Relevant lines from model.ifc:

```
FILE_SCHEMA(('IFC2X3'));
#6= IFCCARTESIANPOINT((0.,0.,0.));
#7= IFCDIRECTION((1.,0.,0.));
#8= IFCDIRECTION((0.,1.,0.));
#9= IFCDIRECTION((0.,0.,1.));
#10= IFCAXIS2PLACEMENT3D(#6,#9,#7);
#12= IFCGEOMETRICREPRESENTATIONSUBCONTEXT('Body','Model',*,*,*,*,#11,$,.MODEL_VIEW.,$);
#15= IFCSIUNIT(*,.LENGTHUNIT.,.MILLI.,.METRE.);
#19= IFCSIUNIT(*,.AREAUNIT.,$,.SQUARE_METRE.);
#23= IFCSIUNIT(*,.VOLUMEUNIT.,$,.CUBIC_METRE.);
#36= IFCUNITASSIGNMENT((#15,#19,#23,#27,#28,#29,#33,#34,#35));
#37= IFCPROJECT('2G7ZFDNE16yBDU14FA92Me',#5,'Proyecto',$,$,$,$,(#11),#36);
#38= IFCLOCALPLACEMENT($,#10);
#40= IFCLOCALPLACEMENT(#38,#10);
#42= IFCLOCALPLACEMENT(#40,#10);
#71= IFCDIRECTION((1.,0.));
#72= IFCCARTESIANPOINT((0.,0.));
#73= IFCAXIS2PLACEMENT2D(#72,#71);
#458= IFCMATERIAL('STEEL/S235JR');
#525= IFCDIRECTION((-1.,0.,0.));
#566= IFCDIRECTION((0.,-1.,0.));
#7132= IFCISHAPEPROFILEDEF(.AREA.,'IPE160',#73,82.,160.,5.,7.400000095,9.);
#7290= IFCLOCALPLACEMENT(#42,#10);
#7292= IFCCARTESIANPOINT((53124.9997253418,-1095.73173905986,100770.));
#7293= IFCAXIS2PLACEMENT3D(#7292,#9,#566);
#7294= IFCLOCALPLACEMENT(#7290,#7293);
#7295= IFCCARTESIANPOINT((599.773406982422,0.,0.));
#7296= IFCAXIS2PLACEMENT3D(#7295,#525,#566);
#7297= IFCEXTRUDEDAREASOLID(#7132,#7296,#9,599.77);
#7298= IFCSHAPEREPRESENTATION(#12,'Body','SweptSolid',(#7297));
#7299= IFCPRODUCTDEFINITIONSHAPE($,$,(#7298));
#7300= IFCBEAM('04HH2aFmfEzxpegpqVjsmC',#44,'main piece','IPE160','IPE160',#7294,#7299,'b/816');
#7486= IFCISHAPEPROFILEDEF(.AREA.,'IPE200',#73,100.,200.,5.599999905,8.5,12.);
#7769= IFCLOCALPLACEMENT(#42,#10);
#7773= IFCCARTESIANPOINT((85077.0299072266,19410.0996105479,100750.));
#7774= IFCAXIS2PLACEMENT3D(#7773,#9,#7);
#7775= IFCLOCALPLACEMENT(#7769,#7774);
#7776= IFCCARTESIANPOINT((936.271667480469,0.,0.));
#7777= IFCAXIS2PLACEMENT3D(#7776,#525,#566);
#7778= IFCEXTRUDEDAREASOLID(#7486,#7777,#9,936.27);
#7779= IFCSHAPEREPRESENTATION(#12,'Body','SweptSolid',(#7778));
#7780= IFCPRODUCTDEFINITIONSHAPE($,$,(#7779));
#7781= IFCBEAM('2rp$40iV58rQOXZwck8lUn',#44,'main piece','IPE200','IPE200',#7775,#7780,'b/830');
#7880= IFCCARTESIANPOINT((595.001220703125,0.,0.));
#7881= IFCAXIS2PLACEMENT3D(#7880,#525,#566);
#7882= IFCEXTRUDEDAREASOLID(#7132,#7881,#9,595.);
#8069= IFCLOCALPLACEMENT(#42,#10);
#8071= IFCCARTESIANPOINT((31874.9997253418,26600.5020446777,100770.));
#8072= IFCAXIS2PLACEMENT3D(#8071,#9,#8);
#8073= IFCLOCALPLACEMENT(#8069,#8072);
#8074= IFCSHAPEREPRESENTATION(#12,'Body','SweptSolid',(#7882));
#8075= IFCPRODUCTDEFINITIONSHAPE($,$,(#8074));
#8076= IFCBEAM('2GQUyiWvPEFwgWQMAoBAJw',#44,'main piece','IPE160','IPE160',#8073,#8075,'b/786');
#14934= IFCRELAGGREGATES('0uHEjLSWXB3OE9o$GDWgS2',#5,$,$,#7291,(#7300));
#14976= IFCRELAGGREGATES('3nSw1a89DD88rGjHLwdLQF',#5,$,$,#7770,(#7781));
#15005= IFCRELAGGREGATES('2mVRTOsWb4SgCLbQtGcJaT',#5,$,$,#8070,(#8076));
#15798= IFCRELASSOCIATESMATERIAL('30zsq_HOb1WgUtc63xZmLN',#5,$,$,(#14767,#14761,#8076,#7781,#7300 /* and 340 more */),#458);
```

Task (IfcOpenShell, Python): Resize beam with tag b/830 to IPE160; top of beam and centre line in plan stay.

```python
import ifcopenshell
import ifcopenshell.util.element
import ifcopenshell.util.representation

model = ifcopenshell.open("model.ifc")

member = model.by_guid("2rp$40iV58rQOXZwck8lUn")
source = next(p for p in model.by_type("IfcIShapeProfileDef") if p.ProfileName == "IPE160")

body = ifcopenshell.util.representation.get_representation(member, "Model", "Body")
solid = body.Items[0]
old_profile = solid.SweptArea

# Copy the section's sizes but keep this member's own profile position.
profile = ifcopenshell.util.element.copy(model, source)
# Profiles are centred, so shift by half the change in depth to hold the top.
shift = (old_profile.OverallDepth - profile.OverallDepth) / 2
x, y = old_profile.Position.Location.Coordinates
up = (0.0, 1.0)  # upwards, in the solid's own plane
location = model.createIfcCartesianPoint((x + up[0] * shift, y + up[1] * shift))
profile.Position = model.createIfcAxis2Placement2D(location, old_profile.Position.RefDirection)
solid.SweptArea = profile
if not model.get_total_inverses(old_profile):
    ifcopenshell.util.element.remove_deep2(model, old_profile)
member.Description = member.Description.replace("IPE200", "IPE160")
member.ObjectType = member.ObjectType.replace("IPE200", "IPE160")

print(solid.SweptArea)

model.write("model_updated.ifc")
```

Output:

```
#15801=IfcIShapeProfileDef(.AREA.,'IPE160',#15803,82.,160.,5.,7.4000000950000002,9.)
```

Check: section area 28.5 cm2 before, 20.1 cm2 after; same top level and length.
